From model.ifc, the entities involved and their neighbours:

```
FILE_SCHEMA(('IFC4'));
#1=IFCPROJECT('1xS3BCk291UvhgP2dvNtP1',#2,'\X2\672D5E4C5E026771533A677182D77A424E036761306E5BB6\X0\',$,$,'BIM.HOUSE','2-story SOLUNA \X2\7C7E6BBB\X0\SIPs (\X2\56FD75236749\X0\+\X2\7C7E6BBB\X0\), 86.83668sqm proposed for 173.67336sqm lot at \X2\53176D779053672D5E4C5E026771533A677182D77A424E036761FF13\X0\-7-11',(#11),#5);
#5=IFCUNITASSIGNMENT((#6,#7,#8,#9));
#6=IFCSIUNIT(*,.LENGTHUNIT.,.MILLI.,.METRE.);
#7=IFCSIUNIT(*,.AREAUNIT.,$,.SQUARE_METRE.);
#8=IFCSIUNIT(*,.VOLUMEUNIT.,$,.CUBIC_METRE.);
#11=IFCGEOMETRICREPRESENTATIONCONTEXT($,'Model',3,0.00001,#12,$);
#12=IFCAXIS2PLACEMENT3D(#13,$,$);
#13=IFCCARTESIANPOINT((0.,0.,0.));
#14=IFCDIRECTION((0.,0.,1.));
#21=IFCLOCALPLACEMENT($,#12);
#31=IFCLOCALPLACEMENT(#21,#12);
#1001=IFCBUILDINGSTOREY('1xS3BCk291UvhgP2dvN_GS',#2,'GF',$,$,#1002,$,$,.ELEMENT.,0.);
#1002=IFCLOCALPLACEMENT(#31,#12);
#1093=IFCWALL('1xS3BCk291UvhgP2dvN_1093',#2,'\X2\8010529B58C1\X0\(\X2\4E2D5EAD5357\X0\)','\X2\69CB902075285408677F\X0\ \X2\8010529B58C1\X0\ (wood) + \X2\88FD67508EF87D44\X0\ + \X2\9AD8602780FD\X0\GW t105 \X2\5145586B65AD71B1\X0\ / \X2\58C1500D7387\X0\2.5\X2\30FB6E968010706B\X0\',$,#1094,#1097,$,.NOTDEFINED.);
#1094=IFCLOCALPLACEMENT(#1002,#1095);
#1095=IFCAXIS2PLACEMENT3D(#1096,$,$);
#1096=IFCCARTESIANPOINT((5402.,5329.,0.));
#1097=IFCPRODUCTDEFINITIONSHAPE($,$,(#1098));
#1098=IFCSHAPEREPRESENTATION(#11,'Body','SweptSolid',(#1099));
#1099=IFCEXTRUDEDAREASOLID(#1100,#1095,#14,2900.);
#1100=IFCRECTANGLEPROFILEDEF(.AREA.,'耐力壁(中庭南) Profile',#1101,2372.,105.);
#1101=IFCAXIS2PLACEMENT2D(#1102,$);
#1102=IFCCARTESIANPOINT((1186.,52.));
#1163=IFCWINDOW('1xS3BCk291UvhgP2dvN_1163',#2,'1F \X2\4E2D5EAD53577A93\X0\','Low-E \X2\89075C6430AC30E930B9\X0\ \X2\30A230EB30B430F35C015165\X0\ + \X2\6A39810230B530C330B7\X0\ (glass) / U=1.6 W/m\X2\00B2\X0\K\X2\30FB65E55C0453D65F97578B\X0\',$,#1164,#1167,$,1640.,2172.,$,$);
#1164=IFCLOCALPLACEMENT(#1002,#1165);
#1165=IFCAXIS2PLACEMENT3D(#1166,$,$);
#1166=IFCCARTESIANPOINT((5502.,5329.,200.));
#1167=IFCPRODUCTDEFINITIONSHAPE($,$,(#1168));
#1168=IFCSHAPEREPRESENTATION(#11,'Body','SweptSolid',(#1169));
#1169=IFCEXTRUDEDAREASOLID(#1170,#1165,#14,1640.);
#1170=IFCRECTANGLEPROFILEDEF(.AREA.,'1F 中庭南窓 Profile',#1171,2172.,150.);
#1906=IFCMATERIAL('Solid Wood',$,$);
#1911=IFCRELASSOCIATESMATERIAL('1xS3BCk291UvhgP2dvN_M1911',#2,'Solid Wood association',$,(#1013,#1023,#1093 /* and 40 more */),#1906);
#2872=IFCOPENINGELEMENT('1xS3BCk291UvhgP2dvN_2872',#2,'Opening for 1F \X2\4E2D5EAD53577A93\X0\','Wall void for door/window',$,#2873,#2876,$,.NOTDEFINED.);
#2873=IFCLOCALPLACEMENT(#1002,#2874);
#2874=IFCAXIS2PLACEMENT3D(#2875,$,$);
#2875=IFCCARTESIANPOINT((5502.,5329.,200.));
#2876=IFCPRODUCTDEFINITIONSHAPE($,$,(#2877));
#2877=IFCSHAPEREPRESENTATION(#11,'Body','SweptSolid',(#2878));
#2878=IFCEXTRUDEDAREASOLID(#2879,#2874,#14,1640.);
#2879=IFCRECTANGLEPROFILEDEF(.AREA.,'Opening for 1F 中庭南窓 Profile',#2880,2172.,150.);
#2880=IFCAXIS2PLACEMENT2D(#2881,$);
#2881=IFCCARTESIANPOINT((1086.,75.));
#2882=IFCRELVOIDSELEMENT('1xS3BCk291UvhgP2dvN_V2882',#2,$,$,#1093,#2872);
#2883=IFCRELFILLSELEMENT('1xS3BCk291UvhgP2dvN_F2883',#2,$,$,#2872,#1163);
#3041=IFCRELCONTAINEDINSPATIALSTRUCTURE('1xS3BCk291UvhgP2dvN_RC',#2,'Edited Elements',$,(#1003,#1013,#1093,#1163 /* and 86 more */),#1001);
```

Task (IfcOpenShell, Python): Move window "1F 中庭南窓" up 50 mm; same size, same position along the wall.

```python
import numpy as np
import ifcopenshell
import ifcopenshell.api.geometry
import ifcopenshell.util.placement
import ifcopenshell.util.unit

model = ifcopenshell.open("model.ifc")
unit_scale = ifcopenshell.util.unit.calculate_unit_scale(model)

window = model.by_guid("1xS3BCk291UvhgP2dvN_1163")
opening = window.FillsVoids[0].RelatingOpeningElement
dz = 0.05 / unit_scale

shift = np.array([0.0, 0.0, dz])
# The window is not placed relative to its opening, so move both.
for product in (opening, window):
    matrix = ifcopenshell.util.placement.get_local_placement(product.ObjectPlacement)
    matrix[:3, 3] += shift
    ifcopenshell.api.geometry.edit_object_placement(model, product=product, matrix=matrix, is_si=False)

print(f"moved by {dz * unit_scale:+.3f} m")

model.write("model-out.ifc")
```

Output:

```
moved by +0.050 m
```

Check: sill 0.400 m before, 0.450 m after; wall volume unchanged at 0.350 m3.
